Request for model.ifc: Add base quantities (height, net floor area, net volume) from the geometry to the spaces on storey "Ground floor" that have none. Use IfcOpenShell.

First a look at what the model holds.

```python
import ifcopenshell
import ifcopenshell.util.element
import ifcopenshell.util.unit

model = ifcopenshell.open("model.ifc")
print(model.schema)
for unit_type in ("LENGTHUNIT", "AREAUNIT", "VOLUMEUNIT"):
    print(unit_type, ifcopenshell.util.unit.calculate_unit_scale(model, unit_type))
storey = next(s for s in model.by_type("IfcBuildingStorey") if s.Name == "Ground floor")
spaces = [e for e in ifcopenshell.util.element.get_decomposition(storey) if e.is_a("IfcSpace")]
for e in sorted(spaces, key=lambda e: e.id()):
    print(e.id(), e.is_a(), e.Name, list(ifcopenshell.util.element.get_psets(e, qtos_only=True)), sep=" | ")
```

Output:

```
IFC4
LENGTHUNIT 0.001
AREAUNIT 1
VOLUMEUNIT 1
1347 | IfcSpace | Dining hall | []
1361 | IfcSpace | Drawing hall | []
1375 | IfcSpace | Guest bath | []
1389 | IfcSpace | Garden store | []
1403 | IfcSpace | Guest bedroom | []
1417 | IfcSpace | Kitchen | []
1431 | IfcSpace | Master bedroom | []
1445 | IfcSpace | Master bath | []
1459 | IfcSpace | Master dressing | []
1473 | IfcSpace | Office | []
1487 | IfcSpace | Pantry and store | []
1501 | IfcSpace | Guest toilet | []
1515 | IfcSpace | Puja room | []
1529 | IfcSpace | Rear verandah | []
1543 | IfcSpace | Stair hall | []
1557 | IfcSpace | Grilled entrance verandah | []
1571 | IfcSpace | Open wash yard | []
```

```python
import ifcopenshell
import ifcopenshell.api.pset
import ifcopenshell.geom
import ifcopenshell.util.element
import ifcopenshell.util.shape
import ifcopenshell.util.unit

model = ifcopenshell.open("model.ifc")
unit_scale = ifcopenshell.util.unit.calculate_unit_scale(model)
area_scale = ifcopenshell.util.unit.calculate_unit_scale(model, "AREAUNIT")
volume_scale = ifcopenshell.util.unit.calculate_unit_scale(model, "VOLUMEUNIT")
settings = ifcopenshell.geom.settings()

storey = next(s for s in model.by_type("IfcBuildingStorey") if s.Name == "Ground floor")
spaces = [e for e in ifcopenshell.util.element.get_decomposition(storey) if e.is_a("IfcSpace")]

for e in sorted(spaces, key=lambda e: e.id()):
    if ifcopenshell.util.element.get_psets(e, qtos_only=True, should_inherit=False):
        continue
    # Geometry comes back in metres, in the element's own axes.
    shape = ifcopenshell.geom.create_shape(settings, e)
    values = {
        "Height": ifcopenshell.util.shape.get_z(shape.geometry) / unit_scale,
        "NetFloorArea": ifcopenshell.util.shape.get_footprint_area(shape.geometry) / area_scale,
        "NetVolume": ifcopenshell.util.shape.get_volume(shape.geometry) / volume_scale,
    }
    qto = ifcopenshell.api.pset.add_qto(model, product=e, name="Qto_SpaceBaseQuantities")
    ifcopenshell.api.pset.edit_qto(model, qto=qto, properties=values)
    print(e.id(), {k: round(v, 3) for k, v in values.items()})

model.write("model-out.ifc")
```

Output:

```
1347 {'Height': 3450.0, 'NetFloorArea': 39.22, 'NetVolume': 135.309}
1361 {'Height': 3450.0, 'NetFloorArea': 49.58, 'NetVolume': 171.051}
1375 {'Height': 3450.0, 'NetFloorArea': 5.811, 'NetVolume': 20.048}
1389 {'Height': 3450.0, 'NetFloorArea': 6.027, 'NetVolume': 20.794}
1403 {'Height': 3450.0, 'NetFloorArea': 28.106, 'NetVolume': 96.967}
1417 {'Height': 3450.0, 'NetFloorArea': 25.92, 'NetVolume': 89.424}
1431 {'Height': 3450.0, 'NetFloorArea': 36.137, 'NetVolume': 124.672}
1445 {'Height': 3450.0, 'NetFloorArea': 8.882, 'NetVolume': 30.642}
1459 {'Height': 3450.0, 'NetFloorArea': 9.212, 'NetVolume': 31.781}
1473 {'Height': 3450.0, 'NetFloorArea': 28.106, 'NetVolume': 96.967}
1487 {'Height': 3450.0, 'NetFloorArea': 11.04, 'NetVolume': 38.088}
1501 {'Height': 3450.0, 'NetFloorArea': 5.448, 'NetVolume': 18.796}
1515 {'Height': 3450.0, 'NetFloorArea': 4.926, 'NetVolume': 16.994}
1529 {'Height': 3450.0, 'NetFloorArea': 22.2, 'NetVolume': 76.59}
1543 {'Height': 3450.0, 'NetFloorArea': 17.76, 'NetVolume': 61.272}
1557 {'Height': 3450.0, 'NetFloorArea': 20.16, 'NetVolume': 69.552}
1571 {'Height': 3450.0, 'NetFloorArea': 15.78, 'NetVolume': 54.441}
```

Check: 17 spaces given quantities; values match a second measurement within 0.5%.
